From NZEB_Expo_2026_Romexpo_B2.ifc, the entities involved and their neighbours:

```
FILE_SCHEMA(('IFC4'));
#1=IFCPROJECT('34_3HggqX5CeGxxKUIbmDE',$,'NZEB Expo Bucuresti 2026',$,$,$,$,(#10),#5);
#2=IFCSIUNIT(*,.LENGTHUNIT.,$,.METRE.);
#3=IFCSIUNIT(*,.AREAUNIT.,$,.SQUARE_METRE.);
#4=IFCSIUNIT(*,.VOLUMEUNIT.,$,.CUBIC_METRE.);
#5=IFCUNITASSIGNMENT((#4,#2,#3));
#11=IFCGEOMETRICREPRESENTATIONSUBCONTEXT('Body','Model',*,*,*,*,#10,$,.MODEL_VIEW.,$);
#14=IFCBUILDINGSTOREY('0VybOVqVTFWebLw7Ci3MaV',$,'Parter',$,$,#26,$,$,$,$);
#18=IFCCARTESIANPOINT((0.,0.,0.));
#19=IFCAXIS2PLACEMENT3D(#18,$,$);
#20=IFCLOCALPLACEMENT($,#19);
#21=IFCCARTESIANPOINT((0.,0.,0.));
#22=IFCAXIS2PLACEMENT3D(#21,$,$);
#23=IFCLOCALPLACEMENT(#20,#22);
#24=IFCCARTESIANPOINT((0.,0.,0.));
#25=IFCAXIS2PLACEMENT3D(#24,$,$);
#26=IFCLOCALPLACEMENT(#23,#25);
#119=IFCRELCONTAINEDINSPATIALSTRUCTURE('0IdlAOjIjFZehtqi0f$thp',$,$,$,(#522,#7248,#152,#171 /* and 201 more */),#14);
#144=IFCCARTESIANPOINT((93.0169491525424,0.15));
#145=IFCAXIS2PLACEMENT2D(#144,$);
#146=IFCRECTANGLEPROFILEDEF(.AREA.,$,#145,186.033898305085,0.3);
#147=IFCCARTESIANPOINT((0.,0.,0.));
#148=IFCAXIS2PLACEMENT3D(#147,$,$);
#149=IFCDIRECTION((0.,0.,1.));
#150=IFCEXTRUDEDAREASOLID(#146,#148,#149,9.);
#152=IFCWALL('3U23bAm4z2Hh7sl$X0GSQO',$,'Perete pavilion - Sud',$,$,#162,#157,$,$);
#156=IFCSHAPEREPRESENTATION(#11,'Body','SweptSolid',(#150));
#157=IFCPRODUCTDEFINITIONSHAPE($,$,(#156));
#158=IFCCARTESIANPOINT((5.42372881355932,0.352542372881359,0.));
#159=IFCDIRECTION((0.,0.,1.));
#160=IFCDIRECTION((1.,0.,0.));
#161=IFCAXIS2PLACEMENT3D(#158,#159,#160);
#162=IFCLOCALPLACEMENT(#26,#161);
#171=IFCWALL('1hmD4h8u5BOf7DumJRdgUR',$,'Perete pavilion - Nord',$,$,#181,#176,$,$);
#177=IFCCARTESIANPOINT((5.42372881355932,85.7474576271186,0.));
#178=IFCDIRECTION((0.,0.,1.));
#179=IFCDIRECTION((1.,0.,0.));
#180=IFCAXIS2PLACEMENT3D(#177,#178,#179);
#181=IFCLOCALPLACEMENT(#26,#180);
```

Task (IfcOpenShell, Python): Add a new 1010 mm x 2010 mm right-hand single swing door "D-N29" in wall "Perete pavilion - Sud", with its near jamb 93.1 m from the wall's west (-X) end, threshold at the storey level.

```python
import numpy as np
import ifcopenshell
import ifcopenshell.api.feature
import ifcopenshell.api.geometry
import ifcopenshell.api.root
import ifcopenshell.api.spatial
import ifcopenshell.geom
import ifcopenshell.util.element
import ifcopenshell.util.placement
import ifcopenshell.util.representation
import ifcopenshell.util.shape
import ifcopenshell.util.unit

model = ifcopenshell.open("NZEB_Expo_2026_Romexpo_B2.ifc")
unit_scale = ifcopenshell.util.unit.calculate_unit_scale(model)
settings = ifcopenshell.geom.settings()


def volume(element):
    """Net volume in cubic metres, openings subtracted."""
    shape = ifcopenshell.geom.create_shape(settings, element)
    return ifcopenshell.util.shape.get_volume(shape.geometry)


wall = model.by_id(152)
storey = ifcopenshell.util.element.get_container(wall, ifc_class="IfcBuildingStorey")
context = ifcopenshell.util.representation.get_context(model, "Model", "Body", "MODEL_VIEW")
before = volume(wall)

width, height, from_end, sill = 1.01, 2.01, 93.1, 0.0  # metres

# The wall runs along its own X axis, and the end named is its -X end.
wall_shape = ifcopenshell.geom.create_shape(settings, wall)
x, y, z = ifcopenshell.util.shape.get_vertices(wall_shape.geometry).T
start = x.min() + from_end
face, thickness = float(y.min()), float(y.max() - y.min())
wall_matrix = ifcopenshell.util.placement.get_local_placement(wall.ObjectPlacement)
level = ifcopenshell.util.placement.get_local_placement(storey.ObjectPlacement)[2, 3]


def in_wall(x, y):
    """Placement at x, y metres in the wall's axes, at sill height."""
    matrix = wall_matrix.copy()
    matrix[:, 3] = wall_matrix @ np.array([x / unit_scale, y / unit_scale, 0.0, 1.0])
    matrix[2, 3] = level + sill / unit_scale
    return matrix


# Opening: a box that overshoots both wall faces by 50 mm.
opening = ifcopenshell.api.root.create_entity(model, ifc_class="IfcOpeningElement", predefined_type="OPENING")
box = ifcopenshell.api.geometry.add_wall_representation(
    model, context=context, length=width, height=height, thickness=thickness + 0.1
)
ifcopenshell.api.geometry.assign_representation(model, product=opening, representation=box)
ifcopenshell.api.geometry.edit_object_placement(model, product=opening, matrix=in_wall(start, face - 0.05), is_si=False)
ifcopenshell.api.feature.add_feature(model, feature=opening, element=wall)

door = ifcopenshell.api.root.create_entity(model, ifc_class="IfcDoor", name="D-N29", predefined_type="DOOR")
door.OverallWidth, door.OverallHeight = width / unit_scale, height / unit_scale
door.OperationType = "SINGLE_SWING_RIGHT"
body = ifcopenshell.api.geometry.add_door_representation(
    model,
    context=context,
    overall_width=door.OverallWidth,
    overall_height=door.OverallHeight,
    operation_type="SINGLE_SWING_RIGHT",
    lining_properties={"LiningDepth": thickness / unit_scale, "ThresholdDepth": thickness / unit_scale},
)
ifcopenshell.api.geometry.assign_representation(model, product=door, representation=body)
ifcopenshell.api.spatial.assign_container(model, products=[door], relating_structure=storey)
ifcopenshell.api.feature.add_filling(model, opening=opening, element=door)

# The lining spans the wall, so the door starts at the wall face.
ifcopenshell.api.geometry.edit_object_placement(model, product=door, matrix=in_wall(start, face), is_si=False)

after = volume(wall)

print(f"wall volume {before:.3f} -> {after:.3f} m3")

model.write("NZEB_Expo_2026_Romexpo_B2-out.ifc")
```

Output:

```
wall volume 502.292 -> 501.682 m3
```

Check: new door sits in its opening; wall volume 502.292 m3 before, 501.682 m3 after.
